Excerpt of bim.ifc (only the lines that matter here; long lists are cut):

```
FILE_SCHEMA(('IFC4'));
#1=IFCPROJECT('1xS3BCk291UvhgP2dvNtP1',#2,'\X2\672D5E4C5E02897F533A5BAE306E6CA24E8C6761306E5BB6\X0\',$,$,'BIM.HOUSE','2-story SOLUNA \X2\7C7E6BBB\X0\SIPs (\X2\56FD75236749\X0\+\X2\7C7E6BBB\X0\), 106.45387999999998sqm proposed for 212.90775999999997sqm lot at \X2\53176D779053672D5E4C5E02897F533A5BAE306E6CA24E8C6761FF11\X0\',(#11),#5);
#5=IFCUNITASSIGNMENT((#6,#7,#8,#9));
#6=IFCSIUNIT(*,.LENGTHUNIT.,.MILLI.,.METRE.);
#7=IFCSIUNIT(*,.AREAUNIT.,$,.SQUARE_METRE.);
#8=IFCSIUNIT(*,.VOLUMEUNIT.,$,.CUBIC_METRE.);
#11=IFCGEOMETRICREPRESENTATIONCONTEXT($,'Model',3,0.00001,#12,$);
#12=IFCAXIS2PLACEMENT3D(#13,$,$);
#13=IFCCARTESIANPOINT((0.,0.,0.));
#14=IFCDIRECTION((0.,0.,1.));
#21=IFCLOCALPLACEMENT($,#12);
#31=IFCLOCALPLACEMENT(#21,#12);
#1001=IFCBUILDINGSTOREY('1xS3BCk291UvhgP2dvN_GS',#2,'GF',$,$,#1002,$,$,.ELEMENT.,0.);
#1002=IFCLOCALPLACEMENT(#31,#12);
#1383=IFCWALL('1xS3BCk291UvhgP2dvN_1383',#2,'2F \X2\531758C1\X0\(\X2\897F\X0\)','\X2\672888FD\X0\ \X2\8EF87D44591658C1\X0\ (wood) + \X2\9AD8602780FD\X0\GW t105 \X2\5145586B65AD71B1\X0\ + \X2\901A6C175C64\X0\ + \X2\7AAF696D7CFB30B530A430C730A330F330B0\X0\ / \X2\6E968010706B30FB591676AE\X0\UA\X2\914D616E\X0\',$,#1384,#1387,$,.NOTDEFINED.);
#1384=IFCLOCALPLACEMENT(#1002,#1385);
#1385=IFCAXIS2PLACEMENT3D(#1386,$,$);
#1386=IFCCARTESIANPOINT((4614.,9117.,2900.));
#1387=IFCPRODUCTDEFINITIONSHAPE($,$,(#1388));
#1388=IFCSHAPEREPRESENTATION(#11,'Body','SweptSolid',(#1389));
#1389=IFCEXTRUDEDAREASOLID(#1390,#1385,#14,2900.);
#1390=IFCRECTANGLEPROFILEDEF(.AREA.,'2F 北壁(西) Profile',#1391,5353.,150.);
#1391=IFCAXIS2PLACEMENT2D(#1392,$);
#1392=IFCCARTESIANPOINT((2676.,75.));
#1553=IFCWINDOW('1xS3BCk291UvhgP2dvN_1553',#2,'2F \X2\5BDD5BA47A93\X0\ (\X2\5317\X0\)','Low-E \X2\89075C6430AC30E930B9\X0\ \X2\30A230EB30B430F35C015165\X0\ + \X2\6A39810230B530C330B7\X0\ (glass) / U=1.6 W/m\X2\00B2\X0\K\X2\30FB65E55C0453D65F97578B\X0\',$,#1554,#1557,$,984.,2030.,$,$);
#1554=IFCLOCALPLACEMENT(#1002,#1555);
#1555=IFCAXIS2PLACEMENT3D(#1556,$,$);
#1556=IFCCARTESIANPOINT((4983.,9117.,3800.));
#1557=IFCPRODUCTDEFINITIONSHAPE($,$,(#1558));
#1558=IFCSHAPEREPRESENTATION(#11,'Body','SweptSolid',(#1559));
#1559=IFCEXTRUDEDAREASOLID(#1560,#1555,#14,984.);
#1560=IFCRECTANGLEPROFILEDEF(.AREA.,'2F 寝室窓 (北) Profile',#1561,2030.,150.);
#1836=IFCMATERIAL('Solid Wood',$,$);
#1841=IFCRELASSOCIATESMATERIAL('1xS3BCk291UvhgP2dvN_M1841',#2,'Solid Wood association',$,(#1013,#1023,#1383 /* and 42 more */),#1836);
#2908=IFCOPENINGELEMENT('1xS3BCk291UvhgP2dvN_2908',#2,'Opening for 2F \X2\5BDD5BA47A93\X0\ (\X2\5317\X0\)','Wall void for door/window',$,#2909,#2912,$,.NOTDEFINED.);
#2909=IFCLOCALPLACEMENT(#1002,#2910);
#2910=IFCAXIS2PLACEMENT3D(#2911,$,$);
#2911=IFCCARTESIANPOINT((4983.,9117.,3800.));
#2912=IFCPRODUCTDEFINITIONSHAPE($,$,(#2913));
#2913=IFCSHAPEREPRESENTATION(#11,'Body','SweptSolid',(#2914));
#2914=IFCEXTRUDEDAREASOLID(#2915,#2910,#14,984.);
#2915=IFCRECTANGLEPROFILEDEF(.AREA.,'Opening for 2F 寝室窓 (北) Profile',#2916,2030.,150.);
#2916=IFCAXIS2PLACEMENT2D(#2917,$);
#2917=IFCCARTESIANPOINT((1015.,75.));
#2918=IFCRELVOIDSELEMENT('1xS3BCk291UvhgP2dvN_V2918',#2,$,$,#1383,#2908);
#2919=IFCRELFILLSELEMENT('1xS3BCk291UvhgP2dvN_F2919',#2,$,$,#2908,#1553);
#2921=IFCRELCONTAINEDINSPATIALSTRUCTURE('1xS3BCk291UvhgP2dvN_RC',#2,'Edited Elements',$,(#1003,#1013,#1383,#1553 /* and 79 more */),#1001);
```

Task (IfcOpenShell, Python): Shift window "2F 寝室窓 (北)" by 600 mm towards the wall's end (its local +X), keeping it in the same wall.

```python
import ifcopenshell
import ifcopenshell.api.geometry
import ifcopenshell.util.placement

model = ifcopenshell.open("bim.ifc")

window = model.by_id(1553)
opening = window.FillsVoids[0].RelatingOpeningElement
wall = opening.VoidsElements[0].RelatingBuildingElement

wall_matrix = ifcopenshell.util.placement.get_local_placement(wall.ObjectPlacement)
shift = wall_matrix[:3, 0] * 600.0
before = ifcopenshell.util.placement.get_local_placement(window.ObjectPlacement)[:3, 3].copy()

# The window is not placed relative to its opening, so move both.
for product in (opening, window):
    matrix = ifcopenshell.util.placement.get_local_placement(product.ObjectPlacement)
    matrix[:3, 3] += shift
    ifcopenshell.api.geometry.edit_object_placement(model, product=product, matrix=matrix, is_si=False)

after = ifcopenshell.util.placement.get_local_placement(window.ObjectPlacement)[:3, 3]
print("window moved by", (after - before).round(3) + 0.0)

model.write("bim-out.ifc")
```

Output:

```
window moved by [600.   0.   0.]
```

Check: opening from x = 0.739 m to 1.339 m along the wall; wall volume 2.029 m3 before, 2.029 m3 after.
